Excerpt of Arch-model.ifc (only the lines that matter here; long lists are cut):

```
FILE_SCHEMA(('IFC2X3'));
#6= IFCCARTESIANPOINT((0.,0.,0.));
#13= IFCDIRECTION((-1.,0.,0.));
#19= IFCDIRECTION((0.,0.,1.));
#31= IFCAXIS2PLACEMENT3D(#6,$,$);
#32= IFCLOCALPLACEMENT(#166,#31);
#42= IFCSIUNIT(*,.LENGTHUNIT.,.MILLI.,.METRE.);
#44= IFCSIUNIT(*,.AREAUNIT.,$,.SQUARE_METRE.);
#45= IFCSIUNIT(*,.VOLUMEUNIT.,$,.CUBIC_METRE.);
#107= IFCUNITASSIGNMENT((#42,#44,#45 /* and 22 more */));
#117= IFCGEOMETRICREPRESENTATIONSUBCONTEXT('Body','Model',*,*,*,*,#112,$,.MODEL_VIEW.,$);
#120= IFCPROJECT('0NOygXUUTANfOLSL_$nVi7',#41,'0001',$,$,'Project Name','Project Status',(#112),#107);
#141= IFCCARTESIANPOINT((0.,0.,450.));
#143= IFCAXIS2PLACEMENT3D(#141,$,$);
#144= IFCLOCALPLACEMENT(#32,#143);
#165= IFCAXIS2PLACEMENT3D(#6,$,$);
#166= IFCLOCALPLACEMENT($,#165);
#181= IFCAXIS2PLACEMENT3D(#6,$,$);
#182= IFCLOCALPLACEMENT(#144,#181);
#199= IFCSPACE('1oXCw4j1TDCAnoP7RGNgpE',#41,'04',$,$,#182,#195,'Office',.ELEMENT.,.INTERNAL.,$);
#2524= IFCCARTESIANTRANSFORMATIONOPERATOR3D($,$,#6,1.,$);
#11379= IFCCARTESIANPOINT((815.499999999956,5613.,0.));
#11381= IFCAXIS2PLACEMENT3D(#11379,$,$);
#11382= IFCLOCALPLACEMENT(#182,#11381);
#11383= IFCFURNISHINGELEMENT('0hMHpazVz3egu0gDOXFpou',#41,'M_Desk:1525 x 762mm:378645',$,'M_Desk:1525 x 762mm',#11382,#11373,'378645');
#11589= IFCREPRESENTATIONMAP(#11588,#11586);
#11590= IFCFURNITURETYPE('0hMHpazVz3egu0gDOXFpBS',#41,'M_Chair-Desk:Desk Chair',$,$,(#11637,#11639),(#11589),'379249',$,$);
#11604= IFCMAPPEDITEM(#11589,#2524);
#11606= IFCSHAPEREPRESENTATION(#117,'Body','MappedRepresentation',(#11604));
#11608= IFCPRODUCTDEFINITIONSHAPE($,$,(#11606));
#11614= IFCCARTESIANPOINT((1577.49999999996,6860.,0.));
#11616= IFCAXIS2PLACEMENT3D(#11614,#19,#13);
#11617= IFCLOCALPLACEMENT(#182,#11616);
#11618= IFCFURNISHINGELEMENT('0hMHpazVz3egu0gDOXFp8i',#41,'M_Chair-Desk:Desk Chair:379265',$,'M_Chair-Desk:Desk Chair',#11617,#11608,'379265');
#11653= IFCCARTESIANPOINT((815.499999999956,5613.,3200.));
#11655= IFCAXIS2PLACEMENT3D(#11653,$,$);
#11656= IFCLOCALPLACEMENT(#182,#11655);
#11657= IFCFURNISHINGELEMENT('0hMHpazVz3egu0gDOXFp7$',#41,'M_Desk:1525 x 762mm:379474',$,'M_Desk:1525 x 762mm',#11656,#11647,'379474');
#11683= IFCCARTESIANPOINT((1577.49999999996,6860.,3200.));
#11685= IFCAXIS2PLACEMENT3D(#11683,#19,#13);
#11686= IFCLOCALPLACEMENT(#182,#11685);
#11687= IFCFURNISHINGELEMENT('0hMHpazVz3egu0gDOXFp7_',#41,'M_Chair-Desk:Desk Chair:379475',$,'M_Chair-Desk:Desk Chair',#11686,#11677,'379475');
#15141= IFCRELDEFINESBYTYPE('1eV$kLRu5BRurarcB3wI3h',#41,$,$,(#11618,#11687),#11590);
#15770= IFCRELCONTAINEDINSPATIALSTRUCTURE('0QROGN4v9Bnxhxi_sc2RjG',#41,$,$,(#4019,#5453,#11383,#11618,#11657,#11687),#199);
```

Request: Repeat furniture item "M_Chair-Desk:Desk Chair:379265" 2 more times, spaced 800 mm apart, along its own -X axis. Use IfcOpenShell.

```python
import ifcopenshell
import ifcopenshell.api.geometry
import ifcopenshell.api.root
import ifcopenshell.util.element
import ifcopenshell.util.placement
import ifcopenshell.util.unit

model = ifcopenshell.open("Arch-model.ifc")
unit_scale = ifcopenshell.util.unit.calculate_unit_scale(model)


def reuse_history(source, copy):
    """copy_class also copies each property set's owner history, people and application; keep the originals."""
    for rel in copy.IsDefinedBy:
        if rel.is_a("IfcRelDefinesByProperties") and (history := rel.RelatingPropertyDefinition.OwnerHistory):
            rel.RelatingPropertyDefinition.OwnerHistory = source.OwnerHistory
            ifcopenshell.util.element.remove_deep2(model, history)


source = model.by_guid("0hMHpazVz3egu0gDOXFp8i")
base = ifcopenshell.util.placement.get_local_placement(source.ObjectPlacement)
step = -base[:3, 0] * 0.8 / unit_scale

for i in range(1, 3):
    copy = ifcopenshell.api.root.copy_class(model, product=source)
    copy.Representation = ifcopenshell.util.element.copy_deep(
        model, source.Representation, exclude=["IfcGeometricRepresentationContext", "IfcRepresentationMap"]
    )
    copy.Name = "M_Chair-Desk:Desk Chair"
    copy.Tag = None
    reuse_history(source, copy)
    matrix = base.copy()
    matrix[:3, 3] += i * step
    print("added at", matrix[:3, 3].round(3) + 0.0)
    ifcopenshell.api.geometry.edit_object_placement(model, product=copy, matrix=matrix, is_si=False)

model.write("Arch-model-out.ifc")
```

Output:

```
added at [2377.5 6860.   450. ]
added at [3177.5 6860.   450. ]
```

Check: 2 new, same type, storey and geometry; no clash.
